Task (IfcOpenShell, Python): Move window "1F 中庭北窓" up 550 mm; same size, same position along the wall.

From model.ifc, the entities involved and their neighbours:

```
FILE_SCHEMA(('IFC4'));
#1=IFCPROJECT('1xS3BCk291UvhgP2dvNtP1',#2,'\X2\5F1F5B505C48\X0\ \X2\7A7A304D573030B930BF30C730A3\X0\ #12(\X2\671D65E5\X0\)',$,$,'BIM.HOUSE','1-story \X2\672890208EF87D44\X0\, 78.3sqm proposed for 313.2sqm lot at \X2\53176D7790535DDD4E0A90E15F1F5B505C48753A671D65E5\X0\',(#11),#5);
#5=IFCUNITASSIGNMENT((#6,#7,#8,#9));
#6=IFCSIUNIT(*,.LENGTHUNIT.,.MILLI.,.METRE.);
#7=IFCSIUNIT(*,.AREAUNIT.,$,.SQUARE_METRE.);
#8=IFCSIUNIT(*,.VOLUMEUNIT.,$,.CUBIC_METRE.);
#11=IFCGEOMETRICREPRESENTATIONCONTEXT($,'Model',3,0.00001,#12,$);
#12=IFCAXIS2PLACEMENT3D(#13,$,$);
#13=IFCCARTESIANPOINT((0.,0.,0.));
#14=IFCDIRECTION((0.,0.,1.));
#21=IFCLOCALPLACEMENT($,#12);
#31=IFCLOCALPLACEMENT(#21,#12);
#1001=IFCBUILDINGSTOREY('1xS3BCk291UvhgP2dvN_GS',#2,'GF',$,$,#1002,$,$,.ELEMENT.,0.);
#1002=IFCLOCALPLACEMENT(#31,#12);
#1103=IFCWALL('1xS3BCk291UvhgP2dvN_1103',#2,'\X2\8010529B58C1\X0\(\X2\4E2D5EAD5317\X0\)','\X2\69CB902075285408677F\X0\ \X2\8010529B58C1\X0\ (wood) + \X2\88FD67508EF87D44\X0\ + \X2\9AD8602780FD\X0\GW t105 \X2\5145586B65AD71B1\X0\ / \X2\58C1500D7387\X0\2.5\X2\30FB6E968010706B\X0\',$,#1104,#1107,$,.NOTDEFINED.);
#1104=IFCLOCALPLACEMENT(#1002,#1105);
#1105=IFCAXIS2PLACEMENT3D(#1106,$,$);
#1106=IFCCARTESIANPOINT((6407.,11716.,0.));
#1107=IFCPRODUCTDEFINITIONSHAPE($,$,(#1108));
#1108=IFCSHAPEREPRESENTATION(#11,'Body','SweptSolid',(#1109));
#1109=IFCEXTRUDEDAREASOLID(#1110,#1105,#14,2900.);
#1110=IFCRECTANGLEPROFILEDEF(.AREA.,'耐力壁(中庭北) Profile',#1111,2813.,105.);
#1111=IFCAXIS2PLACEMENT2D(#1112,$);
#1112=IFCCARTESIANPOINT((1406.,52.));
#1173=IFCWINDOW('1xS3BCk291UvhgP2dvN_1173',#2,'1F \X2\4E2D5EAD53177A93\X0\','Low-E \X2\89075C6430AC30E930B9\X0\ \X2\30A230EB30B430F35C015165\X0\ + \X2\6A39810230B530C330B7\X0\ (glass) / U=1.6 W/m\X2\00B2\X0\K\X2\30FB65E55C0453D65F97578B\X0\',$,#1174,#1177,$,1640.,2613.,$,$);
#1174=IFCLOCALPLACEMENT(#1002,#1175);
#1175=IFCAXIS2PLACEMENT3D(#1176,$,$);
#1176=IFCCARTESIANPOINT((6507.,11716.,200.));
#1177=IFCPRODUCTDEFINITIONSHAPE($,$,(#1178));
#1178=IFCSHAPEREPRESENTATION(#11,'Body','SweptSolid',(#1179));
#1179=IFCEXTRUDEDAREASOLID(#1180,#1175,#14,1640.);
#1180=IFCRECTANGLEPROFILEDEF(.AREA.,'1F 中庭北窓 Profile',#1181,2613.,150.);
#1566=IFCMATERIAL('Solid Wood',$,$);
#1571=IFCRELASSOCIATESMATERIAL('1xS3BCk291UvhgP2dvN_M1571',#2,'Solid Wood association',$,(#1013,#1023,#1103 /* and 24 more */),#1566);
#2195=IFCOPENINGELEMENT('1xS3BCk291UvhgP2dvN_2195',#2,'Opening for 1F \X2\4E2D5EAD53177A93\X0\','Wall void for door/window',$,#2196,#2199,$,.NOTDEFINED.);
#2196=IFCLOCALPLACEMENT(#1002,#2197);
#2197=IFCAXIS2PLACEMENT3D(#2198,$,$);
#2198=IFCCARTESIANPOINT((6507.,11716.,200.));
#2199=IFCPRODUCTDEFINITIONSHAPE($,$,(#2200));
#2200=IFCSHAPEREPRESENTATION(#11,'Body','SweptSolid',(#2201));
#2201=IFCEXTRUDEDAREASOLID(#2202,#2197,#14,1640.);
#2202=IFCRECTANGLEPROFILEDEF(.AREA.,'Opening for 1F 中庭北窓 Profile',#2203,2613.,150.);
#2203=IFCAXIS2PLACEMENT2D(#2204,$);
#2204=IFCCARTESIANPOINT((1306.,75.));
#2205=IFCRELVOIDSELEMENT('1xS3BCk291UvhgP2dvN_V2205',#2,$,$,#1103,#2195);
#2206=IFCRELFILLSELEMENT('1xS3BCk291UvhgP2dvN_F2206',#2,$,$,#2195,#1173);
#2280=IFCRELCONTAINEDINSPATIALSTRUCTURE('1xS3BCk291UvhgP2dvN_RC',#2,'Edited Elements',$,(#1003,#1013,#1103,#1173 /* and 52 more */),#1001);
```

```python
import numpy as np
import ifcopenshell
import ifcopenshell.api.geometry
import ifcopenshell.util.placement
import ifcopenshell.util.unit

model = ifcopenshell.open("model.ifc")
unit_scale = ifcopenshell.util.unit.calculate_unit_scale(model)

window = model.by_guid("1xS3BCk291UvhgP2dvN_1173")
opening = window.FillsVoids[0].RelatingOpeningElement
dz = 550.0

shift = np.array([0.0, 0.0, dz])
# The window is not placed relative to its opening, so move both.
for product in (opening, window):
    matrix = ifcopenshell.util.placement.get_local_placement(product.ObjectPlacement)
    matrix[:3, 3] += shift
    ifcopenshell.api.geometry.edit_object_placement(model, product=product, matrix=matrix, is_si=False)

print(f"moved by {dz * unit_scale:+.3f} m")

model.write("model-out.ifc")
```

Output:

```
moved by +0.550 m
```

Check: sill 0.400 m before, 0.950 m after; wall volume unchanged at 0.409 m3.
